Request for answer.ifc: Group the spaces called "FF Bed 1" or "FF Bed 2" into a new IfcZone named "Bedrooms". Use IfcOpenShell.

First a look at what the model holds.

```python
import ifcopenshell

model = ifcopenshell.open("answer.ifc")
print(model.schema)
seen = {}
for space in model.by_type("IfcSpace"):
    seen[space.Name] = seen.get(space.Name, 0) + 1
for name, count in sorted(seen.items(), key=str):
    print(count, "x", name)
print("zones:", [z.Name for z in model.by_type("IfcZone")][:20])
```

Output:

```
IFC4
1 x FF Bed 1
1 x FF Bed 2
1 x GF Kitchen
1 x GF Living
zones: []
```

```python
import ifcopenshell
import ifcopenshell.api.group
import ifcopenshell.api.root

model = ifcopenshell.open("answer.ifc")

names = {"FF Bed 1", "FF Bed 2"}
spaces = [s for s in model.by_type("IfcSpace") if s.Name in names]

zone = ifcopenshell.api.root.create_entity(model, ifc_class="IfcZone", name="Bedrooms")
ifcopenshell.api.group.assign_group(model, products=spaces, group=zone)
print(len(spaces), "spaces in", zone.Name)

model.write("answer_edited.ifc")
```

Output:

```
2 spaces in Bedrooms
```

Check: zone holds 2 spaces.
